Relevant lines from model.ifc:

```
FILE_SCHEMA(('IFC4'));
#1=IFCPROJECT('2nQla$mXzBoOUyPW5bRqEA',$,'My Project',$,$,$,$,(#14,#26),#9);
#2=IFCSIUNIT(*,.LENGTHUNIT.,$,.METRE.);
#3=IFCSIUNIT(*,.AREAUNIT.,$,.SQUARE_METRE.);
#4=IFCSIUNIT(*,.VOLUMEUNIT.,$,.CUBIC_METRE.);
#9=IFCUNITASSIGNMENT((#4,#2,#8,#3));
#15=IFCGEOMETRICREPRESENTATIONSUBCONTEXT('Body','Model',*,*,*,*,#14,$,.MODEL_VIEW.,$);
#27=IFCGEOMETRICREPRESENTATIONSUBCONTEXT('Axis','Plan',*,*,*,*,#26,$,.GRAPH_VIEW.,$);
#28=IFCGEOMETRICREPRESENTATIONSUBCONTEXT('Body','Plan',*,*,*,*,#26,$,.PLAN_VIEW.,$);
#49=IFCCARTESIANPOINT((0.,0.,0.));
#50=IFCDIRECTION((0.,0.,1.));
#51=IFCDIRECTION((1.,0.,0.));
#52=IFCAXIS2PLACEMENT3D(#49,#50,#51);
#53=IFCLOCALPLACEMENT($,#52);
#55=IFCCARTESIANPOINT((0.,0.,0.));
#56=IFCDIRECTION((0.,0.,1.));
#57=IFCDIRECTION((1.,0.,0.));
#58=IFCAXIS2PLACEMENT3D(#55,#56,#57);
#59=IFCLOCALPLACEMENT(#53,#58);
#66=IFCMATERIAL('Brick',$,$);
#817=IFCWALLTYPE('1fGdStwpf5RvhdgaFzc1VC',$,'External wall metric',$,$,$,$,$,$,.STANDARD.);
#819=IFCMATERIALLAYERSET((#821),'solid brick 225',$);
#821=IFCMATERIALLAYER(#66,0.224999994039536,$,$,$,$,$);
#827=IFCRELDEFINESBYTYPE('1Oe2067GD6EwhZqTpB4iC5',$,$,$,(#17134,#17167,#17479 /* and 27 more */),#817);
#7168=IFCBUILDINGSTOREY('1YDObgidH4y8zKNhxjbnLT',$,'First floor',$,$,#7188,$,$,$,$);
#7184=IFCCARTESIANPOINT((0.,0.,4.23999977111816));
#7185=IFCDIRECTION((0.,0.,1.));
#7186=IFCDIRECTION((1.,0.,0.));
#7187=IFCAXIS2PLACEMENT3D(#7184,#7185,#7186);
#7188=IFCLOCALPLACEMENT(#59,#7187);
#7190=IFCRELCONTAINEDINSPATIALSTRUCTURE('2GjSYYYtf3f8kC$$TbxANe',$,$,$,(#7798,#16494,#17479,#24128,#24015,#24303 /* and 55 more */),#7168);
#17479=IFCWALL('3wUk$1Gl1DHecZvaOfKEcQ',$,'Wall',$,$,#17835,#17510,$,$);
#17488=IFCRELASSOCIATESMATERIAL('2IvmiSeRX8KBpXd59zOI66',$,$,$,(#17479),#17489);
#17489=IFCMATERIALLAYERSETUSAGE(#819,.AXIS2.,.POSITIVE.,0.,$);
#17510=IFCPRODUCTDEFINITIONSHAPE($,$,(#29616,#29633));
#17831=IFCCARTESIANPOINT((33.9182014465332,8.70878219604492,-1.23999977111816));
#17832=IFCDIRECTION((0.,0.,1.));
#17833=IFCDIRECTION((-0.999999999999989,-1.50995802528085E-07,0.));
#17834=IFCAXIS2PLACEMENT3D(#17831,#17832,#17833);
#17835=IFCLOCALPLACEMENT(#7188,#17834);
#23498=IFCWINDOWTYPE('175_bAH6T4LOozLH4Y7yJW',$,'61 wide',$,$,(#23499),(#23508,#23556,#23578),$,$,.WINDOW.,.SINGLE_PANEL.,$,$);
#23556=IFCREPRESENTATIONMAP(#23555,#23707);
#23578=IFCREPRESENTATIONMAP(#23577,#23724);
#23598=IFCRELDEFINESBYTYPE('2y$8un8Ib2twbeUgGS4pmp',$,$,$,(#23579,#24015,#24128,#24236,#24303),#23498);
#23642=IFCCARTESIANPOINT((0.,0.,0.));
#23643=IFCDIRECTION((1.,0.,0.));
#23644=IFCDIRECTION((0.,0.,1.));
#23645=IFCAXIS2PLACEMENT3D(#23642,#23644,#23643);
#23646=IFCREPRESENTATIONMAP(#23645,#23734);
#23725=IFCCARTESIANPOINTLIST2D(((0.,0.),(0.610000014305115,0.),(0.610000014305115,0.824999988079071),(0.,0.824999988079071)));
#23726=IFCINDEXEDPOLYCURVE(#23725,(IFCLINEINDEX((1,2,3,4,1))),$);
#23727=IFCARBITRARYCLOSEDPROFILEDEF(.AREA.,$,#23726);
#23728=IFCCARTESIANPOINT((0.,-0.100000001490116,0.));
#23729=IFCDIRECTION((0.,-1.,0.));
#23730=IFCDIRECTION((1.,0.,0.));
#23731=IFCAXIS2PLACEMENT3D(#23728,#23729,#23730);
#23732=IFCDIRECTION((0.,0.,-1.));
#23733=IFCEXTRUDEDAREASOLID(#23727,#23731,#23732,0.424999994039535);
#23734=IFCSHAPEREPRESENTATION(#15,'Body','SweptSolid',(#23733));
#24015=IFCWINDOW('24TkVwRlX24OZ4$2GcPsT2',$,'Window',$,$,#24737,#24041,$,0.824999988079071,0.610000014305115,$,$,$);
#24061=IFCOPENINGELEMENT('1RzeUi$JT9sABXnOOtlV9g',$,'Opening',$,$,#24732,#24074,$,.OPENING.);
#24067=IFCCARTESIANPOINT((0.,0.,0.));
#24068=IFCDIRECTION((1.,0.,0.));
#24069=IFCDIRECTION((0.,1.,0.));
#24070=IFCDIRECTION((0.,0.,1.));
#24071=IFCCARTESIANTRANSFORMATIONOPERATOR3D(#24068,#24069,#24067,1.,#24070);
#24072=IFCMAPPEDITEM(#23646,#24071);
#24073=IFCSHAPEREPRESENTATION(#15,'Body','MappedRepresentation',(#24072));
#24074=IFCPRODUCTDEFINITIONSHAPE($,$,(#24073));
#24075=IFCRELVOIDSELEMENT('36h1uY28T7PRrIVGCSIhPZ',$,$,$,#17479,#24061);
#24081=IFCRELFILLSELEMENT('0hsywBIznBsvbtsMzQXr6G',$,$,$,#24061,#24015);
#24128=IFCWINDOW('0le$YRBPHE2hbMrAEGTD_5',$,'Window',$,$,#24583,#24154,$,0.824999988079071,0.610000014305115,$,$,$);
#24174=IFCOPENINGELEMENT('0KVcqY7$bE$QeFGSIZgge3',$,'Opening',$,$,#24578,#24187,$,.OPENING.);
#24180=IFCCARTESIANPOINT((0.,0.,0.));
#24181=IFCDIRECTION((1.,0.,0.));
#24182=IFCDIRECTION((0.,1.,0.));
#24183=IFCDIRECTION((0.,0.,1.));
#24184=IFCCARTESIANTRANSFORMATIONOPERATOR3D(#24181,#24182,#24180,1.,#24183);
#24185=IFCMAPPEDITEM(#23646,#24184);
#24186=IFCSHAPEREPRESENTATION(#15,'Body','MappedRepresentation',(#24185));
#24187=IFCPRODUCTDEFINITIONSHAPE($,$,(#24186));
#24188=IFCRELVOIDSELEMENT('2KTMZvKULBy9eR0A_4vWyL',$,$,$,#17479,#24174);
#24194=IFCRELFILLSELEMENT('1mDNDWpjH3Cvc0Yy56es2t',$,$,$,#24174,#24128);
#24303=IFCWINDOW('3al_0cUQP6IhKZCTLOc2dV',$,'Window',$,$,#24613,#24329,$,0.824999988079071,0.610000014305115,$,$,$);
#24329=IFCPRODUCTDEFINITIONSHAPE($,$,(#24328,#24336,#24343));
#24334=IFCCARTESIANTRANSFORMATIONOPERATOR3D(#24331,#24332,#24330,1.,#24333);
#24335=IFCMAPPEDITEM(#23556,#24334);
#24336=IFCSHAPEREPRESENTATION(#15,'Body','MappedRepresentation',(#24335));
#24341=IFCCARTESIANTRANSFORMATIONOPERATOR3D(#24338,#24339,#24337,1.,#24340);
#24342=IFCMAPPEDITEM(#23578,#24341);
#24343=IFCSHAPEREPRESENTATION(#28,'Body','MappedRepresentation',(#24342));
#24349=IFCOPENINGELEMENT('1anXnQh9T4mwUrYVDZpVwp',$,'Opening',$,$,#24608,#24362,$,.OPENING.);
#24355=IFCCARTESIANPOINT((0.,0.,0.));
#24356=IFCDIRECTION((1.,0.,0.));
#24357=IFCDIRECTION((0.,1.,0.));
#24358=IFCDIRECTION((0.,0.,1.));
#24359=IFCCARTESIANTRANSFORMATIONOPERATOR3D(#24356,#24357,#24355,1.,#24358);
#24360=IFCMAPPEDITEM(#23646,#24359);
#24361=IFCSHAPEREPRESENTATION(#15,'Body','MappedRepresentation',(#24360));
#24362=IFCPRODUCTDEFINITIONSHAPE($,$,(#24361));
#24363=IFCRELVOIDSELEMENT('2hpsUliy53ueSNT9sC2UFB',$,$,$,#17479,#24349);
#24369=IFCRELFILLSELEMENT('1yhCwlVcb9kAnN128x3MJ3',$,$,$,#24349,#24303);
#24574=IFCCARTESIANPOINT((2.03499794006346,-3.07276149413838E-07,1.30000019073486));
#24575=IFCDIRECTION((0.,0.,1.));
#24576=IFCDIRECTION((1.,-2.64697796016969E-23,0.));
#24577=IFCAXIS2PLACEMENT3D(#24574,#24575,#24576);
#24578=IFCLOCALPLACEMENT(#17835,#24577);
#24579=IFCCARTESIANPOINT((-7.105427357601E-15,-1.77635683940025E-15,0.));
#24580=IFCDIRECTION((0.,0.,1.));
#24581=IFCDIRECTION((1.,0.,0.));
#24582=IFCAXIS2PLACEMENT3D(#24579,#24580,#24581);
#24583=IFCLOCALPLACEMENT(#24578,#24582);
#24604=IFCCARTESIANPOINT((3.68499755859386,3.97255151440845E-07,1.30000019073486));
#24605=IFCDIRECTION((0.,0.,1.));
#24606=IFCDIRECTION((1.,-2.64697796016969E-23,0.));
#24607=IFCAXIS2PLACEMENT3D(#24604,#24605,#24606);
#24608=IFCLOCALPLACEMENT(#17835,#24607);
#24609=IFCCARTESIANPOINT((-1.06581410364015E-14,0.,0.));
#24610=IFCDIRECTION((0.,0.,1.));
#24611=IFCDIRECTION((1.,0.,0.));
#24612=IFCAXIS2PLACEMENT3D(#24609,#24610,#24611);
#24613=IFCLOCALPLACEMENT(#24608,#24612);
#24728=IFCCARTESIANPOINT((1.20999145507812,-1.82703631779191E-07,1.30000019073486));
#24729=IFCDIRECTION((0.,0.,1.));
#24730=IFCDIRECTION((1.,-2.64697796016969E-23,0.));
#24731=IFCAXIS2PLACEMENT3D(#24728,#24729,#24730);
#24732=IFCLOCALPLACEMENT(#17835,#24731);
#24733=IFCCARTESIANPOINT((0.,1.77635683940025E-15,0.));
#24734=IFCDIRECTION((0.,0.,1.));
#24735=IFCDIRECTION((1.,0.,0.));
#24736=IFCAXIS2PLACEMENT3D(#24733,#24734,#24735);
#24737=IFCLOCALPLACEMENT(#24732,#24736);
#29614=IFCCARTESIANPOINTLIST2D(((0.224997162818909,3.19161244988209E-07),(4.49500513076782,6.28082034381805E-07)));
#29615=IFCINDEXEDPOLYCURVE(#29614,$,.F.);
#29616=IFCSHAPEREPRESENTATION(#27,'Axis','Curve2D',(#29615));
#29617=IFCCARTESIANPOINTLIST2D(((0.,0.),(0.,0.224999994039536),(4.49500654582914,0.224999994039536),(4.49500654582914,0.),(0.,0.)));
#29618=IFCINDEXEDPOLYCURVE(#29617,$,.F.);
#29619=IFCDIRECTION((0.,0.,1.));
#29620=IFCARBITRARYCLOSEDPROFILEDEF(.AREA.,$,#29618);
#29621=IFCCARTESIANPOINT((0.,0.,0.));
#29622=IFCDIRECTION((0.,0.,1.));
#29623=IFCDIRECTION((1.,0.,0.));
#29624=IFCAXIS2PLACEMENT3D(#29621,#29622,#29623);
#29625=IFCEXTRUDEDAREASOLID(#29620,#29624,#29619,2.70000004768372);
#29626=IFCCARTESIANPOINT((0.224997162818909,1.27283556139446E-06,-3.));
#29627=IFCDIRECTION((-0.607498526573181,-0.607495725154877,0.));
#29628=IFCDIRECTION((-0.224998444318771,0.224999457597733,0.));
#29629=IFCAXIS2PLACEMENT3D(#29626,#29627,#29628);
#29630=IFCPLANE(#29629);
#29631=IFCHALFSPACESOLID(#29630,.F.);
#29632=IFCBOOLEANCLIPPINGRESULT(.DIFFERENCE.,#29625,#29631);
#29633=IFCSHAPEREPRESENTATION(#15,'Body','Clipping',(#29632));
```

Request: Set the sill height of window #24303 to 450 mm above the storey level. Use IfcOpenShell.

```python
import numpy as np
import ifcopenshell
import ifcopenshell.api.geometry
import ifcopenshell.geom
import ifcopenshell.util.element
import ifcopenshell.util.placement
import ifcopenshell.util.shape
import ifcopenshell.util.unit

model = ifcopenshell.open("model.ifc")
unit_scale = ifcopenshell.util.unit.calculate_unit_scale(model)

window = model.by_id(24303)
opening = window.FillsVoids[0].RelatingOpeningElement
storey = ifcopenshell.util.element.get_container(window, ifc_class="IfcBuildingStorey")
level = ifcopenshell.util.placement.get_local_placement(storey.ObjectPlacement)[2, 3]

# The opening's origin need not be at the sill, so measure its lowest point.
shape = ifcopenshell.geom.create_shape(ifcopenshell.geom.settings(), opening)
bottom = ifcopenshell.util.shape.get_shape_bottom_elevation(shape, shape.geometry) / unit_scale
dz = level + 0.45 - bottom

shift = np.array([0.0, 0.0, dz])
# The window is placed relative to its opening, so it follows when the opening moves.
matrix = ifcopenshell.util.placement.get_local_placement(opening.ObjectPlacement)
matrix[:3, 3] += shift
ifcopenshell.api.geometry.edit_object_placement(
    model, product=opening, matrix=matrix, is_si=False, should_transform_children=True
)

print(f"moved by {dz * unit_scale:+.3f} m")

model.write("model_edited.ifc")
```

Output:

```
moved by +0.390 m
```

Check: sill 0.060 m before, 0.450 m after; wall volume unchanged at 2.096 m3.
